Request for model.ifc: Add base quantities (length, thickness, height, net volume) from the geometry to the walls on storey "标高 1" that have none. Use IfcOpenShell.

First a look at what the model holds.

```python
import ifcopenshell
import ifcopenshell.util.element
import ifcopenshell.util.unit

model = ifcopenshell.open("model.ifc")
print(model.schema)
for unit_type in ("LENGTHUNIT", "AREAUNIT", "VOLUMEUNIT"):
    print(unit_type, ifcopenshell.util.unit.calculate_unit_scale(model, unit_type))
storey = next(s for s in model.by_type("IfcBuildingStorey") if s.Name == "标高 1")
walls = [e for e in ifcopenshell.util.element.get_decomposition(storey) if e.is_a("IfcWall")]
for e in sorted(walls, key=lambda e: e.id()):
    print(e.id(), e.is_a(), e.Name, list(ifcopenshell.util.element.get_psets(e, qtos_only=True)), sep=" | ")
```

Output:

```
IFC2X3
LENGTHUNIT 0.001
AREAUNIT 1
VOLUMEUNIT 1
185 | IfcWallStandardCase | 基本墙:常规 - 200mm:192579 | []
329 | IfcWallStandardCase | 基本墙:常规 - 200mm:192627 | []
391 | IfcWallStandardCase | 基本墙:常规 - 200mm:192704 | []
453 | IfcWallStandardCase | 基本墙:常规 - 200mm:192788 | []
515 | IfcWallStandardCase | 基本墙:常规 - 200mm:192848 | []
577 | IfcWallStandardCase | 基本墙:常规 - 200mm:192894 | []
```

```python
import ifcopenshell
import ifcopenshell.api.pset
import ifcopenshell.geom
import ifcopenshell.util.element
import ifcopenshell.util.shape
import ifcopenshell.util.unit

model = ifcopenshell.open("model.ifc")
unit_scale = ifcopenshell.util.unit.calculate_unit_scale(model)
volume_scale = ifcopenshell.util.unit.calculate_unit_scale(model, "VOLUMEUNIT")
settings = ifcopenshell.geom.settings()

storey = next(s for s in model.by_type("IfcBuildingStorey") if s.Name == "标高 1")
walls = [e for e in ifcopenshell.util.element.get_decomposition(storey) if e.is_a("IfcWall")]

for e in sorted(walls, key=lambda e: e.id()):
    if ifcopenshell.util.element.get_psets(e, qtos_only=True, should_inherit=False):
        continue
    # Geometry comes back in metres, in the element's own axes.
    shape = ifcopenshell.geom.create_shape(settings, e)
    values = {
        "Length": ifcopenshell.util.shape.get_x(shape.geometry) / unit_scale,
        "Width": ifcopenshell.util.shape.get_y(shape.geometry) / unit_scale,
        "Height": ifcopenshell.util.shape.get_z(shape.geometry) / unit_scale,
        "NetVolume": ifcopenshell.util.shape.get_volume(shape.geometry) / volume_scale,
    }
    qto = ifcopenshell.api.pset.add_qto(model, product=e, name="BaseQuantities")
    ifcopenshell.api.pset.edit_qto(model, qto=qto, properties=values)
    print(e.id(), {k: round(v, 3) for k, v in values.items()})

model.write("model_edited.ifc")
```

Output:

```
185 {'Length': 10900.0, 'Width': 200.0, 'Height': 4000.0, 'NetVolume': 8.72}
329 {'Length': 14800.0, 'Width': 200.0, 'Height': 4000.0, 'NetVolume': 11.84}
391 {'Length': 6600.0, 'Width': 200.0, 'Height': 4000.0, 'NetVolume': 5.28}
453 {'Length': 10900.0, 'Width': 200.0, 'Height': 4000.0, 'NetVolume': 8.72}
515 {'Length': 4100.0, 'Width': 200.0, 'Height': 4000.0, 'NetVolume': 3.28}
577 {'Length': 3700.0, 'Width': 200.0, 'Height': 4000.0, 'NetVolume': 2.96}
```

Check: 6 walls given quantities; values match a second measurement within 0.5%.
